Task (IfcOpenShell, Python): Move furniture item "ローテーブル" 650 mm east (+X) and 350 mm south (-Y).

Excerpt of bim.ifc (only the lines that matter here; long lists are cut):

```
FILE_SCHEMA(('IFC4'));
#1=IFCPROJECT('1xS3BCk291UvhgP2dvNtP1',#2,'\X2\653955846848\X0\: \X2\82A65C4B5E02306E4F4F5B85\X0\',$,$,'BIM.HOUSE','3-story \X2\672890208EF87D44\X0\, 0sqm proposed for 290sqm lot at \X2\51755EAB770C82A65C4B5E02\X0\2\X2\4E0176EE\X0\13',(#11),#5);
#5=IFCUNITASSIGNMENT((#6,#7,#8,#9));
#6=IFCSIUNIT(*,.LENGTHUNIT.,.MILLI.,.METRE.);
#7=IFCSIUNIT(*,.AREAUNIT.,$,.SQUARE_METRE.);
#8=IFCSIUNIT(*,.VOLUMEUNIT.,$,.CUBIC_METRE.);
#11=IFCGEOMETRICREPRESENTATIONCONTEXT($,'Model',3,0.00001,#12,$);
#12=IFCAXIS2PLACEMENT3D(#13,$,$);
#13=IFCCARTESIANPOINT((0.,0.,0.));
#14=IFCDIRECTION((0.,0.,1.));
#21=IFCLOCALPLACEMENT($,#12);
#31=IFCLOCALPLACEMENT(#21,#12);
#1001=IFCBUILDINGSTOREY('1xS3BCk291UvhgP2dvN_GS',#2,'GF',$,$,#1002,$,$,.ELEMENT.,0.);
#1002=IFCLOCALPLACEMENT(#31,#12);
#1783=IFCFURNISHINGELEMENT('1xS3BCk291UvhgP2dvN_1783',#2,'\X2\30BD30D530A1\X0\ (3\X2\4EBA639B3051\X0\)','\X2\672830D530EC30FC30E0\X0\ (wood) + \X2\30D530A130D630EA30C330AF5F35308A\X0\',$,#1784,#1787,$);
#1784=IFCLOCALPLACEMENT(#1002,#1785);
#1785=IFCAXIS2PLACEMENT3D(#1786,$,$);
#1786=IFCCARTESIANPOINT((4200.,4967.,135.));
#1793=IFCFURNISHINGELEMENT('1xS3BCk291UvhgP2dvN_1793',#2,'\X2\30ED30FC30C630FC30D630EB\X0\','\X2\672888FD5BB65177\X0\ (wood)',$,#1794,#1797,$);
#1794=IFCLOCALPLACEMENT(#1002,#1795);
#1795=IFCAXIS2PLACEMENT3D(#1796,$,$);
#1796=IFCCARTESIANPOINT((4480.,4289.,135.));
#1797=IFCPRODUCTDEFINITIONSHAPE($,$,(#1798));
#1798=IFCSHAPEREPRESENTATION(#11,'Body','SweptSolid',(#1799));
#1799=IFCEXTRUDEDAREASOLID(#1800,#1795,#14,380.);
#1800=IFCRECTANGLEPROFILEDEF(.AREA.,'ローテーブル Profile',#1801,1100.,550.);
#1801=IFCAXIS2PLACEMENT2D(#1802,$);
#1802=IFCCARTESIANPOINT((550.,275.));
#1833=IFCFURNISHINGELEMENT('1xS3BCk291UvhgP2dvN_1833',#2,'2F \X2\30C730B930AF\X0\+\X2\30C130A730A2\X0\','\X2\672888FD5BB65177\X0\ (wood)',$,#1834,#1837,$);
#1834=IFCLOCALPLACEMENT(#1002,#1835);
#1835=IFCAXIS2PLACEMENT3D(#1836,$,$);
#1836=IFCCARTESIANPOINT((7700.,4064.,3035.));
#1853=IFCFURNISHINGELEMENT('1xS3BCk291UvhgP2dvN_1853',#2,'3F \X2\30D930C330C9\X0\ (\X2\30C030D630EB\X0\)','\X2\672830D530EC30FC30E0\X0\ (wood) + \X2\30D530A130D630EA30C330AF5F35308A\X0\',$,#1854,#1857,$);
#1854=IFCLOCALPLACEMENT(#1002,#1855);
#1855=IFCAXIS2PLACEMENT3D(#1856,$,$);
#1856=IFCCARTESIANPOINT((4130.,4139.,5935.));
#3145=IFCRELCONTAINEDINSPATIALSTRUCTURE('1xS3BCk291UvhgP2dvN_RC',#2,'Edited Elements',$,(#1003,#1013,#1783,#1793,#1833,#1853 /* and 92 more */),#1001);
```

```python
import ifcopenshell
import ifcopenshell.api.geometry
import ifcopenshell.util.placement
import ifcopenshell.util.unit

model = ifcopenshell.open("bim.ifc")
unit_scale = ifcopenshell.util.unit.calculate_unit_scale(model)

item = model.by_id(1793)
matrix = ifcopenshell.util.placement.get_local_placement(item.ObjectPlacement)
matrix[0, 3] += 0.65 / unit_scale
matrix[1, 3] -= 0.35 / unit_scale
ifcopenshell.api.geometry.edit_object_placement(model, product=item, matrix=matrix, is_si=False)

print(ifcopenshell.util.placement.get_local_placement(item.ObjectPlacement).round(3) + 0.0)

model.write("bim-out.ifc")
```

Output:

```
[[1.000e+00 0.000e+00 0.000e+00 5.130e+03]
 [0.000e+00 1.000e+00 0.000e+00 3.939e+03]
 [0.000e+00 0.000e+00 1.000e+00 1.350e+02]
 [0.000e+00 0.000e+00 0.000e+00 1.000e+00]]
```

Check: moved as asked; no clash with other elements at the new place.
